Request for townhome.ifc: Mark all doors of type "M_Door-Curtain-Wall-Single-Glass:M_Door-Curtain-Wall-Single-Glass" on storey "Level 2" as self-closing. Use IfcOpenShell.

First a look at what the model holds.

```python
import ifcopenshell
import ifcopenshell.util.element

model = ifcopenshell.open("townhome.ifc")
print(model.schema)
storey = next(s for s in model.by_type("IfcBuildingStorey") if s.Name == "Level 2")
doors = [e for e in ifcopenshell.util.element.get_decomposition(storey) if e.is_a("IfcDoor")]
seen = {}
for e in doors:
    element_type = ifcopenshell.util.element.get_type(e)
    key = (element_type.Name if element_type != e and element_type else None, ifcopenshell.util.element.get_pset(e, "Pset_DoorCommon", "SelfClosing"))
    seen[key] = seen.get(key, 0) + 1
for (name, value), count in sorted(seen.items(), key=str):
    print(count, "x", name, "|", value)
```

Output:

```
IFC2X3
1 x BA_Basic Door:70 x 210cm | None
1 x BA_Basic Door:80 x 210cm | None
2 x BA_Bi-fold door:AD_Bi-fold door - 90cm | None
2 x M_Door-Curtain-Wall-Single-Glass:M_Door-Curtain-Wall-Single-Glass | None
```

```python
import ifcopenshell
import ifcopenshell.api.pset
import ifcopenshell.util.element

model = ifcopenshell.open("townhome.ifc")

storey = next(s for s in model.by_type("IfcBuildingStorey") if s.Name == "Level 2")
doors = [e for e in ifcopenshell.util.element.get_decomposition(storey) if e.is_a("IfcDoor")]

count = 0
for e in doors:
    element_type = ifcopenshell.util.element.get_type(e)
    if element_type in (None, e) or element_type.Name != "M_Door-Curtain-Wall-Single-Glass:M_Door-Curtain-Wall-Single-Glass":
        continue
    # add_pset returns the element's existing set when there is one.
    pset = ifcopenshell.api.pset.add_pset(model, product=e, name="Pset_DoorCommon")
    ifcopenshell.api.pset.edit_pset(model, pset=pset, properties={"SelfClosing": True})
    count += 1

print(count, "doors updated")

model.write("townhome_edited.ifc")
```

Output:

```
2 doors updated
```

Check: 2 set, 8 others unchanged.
